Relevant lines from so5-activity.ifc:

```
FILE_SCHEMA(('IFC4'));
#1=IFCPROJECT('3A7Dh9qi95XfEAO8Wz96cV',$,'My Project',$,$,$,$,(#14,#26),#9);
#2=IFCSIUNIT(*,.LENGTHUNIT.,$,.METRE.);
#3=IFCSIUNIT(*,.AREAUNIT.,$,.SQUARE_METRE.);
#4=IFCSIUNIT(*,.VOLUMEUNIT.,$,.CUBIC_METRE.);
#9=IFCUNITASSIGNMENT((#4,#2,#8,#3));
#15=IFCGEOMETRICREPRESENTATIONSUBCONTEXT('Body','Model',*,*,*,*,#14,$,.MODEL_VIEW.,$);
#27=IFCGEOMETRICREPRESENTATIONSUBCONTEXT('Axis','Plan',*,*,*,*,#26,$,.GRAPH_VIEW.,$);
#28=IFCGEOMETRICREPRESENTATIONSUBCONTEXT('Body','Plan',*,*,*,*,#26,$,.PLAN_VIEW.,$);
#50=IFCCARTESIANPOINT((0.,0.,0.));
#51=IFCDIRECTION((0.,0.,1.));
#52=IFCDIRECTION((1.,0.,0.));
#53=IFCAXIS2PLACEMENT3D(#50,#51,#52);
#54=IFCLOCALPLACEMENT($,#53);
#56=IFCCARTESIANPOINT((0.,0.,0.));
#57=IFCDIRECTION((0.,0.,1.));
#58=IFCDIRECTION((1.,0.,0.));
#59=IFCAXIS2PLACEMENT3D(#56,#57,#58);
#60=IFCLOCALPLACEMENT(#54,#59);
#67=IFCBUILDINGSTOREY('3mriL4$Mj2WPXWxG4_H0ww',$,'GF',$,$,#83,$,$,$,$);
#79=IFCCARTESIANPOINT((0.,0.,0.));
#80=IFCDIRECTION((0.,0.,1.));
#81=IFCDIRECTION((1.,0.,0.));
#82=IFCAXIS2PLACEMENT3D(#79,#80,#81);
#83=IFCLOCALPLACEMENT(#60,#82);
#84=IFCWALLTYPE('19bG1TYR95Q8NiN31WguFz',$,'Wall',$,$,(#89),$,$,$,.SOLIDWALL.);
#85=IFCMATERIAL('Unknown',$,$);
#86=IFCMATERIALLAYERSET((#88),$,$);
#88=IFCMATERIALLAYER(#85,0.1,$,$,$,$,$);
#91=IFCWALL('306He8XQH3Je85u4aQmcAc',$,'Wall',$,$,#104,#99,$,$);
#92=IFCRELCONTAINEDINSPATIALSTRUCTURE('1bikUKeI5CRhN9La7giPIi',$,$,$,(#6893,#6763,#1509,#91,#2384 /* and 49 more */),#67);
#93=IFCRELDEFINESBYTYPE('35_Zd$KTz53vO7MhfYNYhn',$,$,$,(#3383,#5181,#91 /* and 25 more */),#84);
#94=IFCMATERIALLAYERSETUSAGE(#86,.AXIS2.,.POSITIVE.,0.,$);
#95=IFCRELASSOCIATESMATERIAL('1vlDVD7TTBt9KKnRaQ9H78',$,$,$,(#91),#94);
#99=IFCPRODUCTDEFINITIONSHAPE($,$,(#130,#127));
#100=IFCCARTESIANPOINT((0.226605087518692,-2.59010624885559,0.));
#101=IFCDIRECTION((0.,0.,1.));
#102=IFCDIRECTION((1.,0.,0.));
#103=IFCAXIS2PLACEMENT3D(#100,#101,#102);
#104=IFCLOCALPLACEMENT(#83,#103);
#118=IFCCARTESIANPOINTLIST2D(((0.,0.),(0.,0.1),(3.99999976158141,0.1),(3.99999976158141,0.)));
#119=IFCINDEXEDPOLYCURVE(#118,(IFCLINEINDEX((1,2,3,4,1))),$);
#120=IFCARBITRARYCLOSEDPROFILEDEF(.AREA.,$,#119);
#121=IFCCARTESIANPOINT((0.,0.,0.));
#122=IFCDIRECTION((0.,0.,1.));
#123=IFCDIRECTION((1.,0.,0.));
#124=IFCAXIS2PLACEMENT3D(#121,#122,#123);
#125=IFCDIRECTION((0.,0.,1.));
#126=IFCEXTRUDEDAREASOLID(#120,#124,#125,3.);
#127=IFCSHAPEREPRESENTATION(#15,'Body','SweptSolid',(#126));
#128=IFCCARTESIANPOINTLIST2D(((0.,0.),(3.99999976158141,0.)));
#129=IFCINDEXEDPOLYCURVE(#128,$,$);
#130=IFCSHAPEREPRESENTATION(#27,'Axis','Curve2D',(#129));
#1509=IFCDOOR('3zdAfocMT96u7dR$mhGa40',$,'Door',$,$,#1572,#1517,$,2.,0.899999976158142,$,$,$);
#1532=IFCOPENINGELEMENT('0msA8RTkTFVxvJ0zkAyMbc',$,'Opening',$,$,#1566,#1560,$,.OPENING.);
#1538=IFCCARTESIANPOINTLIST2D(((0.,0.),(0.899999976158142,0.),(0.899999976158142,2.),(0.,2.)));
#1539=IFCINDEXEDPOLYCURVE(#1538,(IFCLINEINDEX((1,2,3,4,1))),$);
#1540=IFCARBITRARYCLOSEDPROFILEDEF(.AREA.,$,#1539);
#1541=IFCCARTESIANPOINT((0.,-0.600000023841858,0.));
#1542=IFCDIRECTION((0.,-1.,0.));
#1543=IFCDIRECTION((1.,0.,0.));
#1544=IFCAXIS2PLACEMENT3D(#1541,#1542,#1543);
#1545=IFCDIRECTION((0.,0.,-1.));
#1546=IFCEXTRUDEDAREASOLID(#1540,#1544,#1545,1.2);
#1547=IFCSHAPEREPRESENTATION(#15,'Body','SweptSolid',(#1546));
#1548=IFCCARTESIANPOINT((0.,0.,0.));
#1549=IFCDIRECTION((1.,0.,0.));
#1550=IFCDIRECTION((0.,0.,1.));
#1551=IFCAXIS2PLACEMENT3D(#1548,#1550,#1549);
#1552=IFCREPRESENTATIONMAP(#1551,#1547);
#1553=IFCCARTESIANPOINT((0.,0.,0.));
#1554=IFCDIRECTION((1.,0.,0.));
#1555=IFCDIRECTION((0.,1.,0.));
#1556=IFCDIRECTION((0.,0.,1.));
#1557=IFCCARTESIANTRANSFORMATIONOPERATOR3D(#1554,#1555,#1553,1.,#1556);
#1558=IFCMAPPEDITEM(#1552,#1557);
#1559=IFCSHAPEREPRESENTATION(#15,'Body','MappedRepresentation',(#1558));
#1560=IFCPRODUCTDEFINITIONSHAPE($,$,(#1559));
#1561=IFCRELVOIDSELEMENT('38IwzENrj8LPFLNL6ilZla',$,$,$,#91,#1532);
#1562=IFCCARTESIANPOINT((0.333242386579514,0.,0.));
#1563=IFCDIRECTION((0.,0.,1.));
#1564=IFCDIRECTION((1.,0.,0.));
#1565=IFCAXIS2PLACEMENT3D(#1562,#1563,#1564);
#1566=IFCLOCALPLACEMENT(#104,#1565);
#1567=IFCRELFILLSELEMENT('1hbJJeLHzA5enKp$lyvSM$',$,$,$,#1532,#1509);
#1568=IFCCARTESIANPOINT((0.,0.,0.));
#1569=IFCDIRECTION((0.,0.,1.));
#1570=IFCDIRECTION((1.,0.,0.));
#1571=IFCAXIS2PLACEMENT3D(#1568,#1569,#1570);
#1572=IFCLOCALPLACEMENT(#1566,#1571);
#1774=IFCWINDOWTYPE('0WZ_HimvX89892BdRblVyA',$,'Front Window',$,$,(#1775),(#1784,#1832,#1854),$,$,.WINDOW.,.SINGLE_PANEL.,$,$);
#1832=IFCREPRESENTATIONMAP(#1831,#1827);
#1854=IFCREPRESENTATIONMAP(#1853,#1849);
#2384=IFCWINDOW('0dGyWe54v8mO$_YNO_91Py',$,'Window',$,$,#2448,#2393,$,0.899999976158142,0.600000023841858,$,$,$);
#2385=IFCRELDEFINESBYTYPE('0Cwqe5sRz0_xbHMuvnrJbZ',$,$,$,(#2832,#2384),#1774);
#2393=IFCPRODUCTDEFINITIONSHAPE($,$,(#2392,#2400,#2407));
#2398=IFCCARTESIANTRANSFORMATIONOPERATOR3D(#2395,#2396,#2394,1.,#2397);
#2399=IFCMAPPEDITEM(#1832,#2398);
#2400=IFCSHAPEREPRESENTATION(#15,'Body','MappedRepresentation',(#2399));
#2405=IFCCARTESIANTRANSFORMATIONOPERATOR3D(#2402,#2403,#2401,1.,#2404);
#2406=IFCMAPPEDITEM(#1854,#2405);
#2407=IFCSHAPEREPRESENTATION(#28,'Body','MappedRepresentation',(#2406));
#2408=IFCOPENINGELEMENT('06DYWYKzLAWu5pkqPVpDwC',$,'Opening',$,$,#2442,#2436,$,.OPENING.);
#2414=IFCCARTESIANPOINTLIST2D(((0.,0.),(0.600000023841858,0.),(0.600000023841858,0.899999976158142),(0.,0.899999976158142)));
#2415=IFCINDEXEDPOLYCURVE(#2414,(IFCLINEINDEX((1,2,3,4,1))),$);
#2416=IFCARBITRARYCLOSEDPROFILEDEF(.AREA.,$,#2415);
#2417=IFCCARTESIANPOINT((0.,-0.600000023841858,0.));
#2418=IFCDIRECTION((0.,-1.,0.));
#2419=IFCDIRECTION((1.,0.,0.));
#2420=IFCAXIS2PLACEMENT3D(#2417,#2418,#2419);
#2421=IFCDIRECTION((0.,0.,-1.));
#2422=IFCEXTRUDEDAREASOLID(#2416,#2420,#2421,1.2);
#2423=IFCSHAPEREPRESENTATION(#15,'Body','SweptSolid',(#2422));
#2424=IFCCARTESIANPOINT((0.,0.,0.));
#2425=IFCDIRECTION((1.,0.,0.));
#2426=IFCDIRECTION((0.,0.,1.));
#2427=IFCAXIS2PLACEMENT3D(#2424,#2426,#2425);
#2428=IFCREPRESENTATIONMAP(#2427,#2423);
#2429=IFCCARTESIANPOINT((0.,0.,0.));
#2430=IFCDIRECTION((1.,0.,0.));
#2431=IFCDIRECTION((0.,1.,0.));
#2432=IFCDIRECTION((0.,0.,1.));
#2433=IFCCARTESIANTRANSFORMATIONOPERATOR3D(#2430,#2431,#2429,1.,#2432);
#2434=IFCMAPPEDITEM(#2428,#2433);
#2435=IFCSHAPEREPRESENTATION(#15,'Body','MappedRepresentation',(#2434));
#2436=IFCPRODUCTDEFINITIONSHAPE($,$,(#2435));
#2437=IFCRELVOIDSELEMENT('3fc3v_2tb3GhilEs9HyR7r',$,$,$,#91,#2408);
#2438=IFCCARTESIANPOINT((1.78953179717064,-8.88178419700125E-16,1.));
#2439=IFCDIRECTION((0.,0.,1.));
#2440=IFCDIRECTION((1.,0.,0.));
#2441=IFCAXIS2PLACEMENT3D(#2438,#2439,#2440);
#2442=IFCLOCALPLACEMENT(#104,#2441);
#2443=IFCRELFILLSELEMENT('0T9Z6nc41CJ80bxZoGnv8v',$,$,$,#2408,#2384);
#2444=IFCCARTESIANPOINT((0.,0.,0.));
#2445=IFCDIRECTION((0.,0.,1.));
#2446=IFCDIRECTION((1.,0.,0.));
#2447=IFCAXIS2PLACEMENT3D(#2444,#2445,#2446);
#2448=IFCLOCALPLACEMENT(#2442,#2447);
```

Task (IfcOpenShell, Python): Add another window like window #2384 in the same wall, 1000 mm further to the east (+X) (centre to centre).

```python
import ifcopenshell
import ifcopenshell.api.feature
import ifcopenshell.api.geometry
import ifcopenshell.api.root
import ifcopenshell.geom
import ifcopenshell.util.element
import ifcopenshell.util.placement
import ifcopenshell.util.shape
import ifcopenshell.util.unit

model = ifcopenshell.open("so5-activity.ifc")
unit_scale = ifcopenshell.util.unit.calculate_unit_scale(model)
settings = ifcopenshell.geom.settings()


def volume(element):
    """Net volume in cubic metres, openings subtracted."""
    shape = ifcopenshell.geom.create_shape(settings, element)
    return ifcopenshell.util.shape.get_volume(shape.geometry)


window = model.by_id(2384)
opening = window.FillsVoids[0].RelatingOpeningElement
wall = opening.VoidsElements[0].RelatingBuildingElement
before = volume(wall)
shift = ifcopenshell.util.placement.get_local_placement(wall.ObjectPlacement)[:3, 0] * 1 / unit_scale

# copy_class copies the void relationship, type, container and properties, but no geometry.
new_opening = ifcopenshell.api.root.copy_class(model, product=opening)
new_opening.Representation = ifcopenshell.util.element.copy_deep(
    model, opening.Representation, exclude=["IfcGeometricRepresentationContext", "IfcRepresentationMap"]
)
new_window = ifcopenshell.api.root.copy_class(model, product=window)
new_window.Representation = ifcopenshell.util.element.copy_deep(
    model, window.Representation, exclude=["IfcGeometricRepresentationContext", "IfcRepresentationMap"]
)
ifcopenshell.api.feature.add_filling(model, opening=new_opening, element=new_window)

for old, new in ((opening, new_opening), (window, new_window)):
    matrix = ifcopenshell.util.placement.get_local_placement(old.ObjectPlacement)
    matrix[:3, 3] += shift
    ifcopenshell.api.geometry.edit_object_placement(model, product=new, matrix=matrix, is_si=False)

after = volume(wall)

print(f"wall volume {before:.3f} -> {after:.3f} m3")

model.write("so5-activity-out.ifc")
```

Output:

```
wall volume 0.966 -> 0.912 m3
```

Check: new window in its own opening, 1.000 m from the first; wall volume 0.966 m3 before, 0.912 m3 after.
